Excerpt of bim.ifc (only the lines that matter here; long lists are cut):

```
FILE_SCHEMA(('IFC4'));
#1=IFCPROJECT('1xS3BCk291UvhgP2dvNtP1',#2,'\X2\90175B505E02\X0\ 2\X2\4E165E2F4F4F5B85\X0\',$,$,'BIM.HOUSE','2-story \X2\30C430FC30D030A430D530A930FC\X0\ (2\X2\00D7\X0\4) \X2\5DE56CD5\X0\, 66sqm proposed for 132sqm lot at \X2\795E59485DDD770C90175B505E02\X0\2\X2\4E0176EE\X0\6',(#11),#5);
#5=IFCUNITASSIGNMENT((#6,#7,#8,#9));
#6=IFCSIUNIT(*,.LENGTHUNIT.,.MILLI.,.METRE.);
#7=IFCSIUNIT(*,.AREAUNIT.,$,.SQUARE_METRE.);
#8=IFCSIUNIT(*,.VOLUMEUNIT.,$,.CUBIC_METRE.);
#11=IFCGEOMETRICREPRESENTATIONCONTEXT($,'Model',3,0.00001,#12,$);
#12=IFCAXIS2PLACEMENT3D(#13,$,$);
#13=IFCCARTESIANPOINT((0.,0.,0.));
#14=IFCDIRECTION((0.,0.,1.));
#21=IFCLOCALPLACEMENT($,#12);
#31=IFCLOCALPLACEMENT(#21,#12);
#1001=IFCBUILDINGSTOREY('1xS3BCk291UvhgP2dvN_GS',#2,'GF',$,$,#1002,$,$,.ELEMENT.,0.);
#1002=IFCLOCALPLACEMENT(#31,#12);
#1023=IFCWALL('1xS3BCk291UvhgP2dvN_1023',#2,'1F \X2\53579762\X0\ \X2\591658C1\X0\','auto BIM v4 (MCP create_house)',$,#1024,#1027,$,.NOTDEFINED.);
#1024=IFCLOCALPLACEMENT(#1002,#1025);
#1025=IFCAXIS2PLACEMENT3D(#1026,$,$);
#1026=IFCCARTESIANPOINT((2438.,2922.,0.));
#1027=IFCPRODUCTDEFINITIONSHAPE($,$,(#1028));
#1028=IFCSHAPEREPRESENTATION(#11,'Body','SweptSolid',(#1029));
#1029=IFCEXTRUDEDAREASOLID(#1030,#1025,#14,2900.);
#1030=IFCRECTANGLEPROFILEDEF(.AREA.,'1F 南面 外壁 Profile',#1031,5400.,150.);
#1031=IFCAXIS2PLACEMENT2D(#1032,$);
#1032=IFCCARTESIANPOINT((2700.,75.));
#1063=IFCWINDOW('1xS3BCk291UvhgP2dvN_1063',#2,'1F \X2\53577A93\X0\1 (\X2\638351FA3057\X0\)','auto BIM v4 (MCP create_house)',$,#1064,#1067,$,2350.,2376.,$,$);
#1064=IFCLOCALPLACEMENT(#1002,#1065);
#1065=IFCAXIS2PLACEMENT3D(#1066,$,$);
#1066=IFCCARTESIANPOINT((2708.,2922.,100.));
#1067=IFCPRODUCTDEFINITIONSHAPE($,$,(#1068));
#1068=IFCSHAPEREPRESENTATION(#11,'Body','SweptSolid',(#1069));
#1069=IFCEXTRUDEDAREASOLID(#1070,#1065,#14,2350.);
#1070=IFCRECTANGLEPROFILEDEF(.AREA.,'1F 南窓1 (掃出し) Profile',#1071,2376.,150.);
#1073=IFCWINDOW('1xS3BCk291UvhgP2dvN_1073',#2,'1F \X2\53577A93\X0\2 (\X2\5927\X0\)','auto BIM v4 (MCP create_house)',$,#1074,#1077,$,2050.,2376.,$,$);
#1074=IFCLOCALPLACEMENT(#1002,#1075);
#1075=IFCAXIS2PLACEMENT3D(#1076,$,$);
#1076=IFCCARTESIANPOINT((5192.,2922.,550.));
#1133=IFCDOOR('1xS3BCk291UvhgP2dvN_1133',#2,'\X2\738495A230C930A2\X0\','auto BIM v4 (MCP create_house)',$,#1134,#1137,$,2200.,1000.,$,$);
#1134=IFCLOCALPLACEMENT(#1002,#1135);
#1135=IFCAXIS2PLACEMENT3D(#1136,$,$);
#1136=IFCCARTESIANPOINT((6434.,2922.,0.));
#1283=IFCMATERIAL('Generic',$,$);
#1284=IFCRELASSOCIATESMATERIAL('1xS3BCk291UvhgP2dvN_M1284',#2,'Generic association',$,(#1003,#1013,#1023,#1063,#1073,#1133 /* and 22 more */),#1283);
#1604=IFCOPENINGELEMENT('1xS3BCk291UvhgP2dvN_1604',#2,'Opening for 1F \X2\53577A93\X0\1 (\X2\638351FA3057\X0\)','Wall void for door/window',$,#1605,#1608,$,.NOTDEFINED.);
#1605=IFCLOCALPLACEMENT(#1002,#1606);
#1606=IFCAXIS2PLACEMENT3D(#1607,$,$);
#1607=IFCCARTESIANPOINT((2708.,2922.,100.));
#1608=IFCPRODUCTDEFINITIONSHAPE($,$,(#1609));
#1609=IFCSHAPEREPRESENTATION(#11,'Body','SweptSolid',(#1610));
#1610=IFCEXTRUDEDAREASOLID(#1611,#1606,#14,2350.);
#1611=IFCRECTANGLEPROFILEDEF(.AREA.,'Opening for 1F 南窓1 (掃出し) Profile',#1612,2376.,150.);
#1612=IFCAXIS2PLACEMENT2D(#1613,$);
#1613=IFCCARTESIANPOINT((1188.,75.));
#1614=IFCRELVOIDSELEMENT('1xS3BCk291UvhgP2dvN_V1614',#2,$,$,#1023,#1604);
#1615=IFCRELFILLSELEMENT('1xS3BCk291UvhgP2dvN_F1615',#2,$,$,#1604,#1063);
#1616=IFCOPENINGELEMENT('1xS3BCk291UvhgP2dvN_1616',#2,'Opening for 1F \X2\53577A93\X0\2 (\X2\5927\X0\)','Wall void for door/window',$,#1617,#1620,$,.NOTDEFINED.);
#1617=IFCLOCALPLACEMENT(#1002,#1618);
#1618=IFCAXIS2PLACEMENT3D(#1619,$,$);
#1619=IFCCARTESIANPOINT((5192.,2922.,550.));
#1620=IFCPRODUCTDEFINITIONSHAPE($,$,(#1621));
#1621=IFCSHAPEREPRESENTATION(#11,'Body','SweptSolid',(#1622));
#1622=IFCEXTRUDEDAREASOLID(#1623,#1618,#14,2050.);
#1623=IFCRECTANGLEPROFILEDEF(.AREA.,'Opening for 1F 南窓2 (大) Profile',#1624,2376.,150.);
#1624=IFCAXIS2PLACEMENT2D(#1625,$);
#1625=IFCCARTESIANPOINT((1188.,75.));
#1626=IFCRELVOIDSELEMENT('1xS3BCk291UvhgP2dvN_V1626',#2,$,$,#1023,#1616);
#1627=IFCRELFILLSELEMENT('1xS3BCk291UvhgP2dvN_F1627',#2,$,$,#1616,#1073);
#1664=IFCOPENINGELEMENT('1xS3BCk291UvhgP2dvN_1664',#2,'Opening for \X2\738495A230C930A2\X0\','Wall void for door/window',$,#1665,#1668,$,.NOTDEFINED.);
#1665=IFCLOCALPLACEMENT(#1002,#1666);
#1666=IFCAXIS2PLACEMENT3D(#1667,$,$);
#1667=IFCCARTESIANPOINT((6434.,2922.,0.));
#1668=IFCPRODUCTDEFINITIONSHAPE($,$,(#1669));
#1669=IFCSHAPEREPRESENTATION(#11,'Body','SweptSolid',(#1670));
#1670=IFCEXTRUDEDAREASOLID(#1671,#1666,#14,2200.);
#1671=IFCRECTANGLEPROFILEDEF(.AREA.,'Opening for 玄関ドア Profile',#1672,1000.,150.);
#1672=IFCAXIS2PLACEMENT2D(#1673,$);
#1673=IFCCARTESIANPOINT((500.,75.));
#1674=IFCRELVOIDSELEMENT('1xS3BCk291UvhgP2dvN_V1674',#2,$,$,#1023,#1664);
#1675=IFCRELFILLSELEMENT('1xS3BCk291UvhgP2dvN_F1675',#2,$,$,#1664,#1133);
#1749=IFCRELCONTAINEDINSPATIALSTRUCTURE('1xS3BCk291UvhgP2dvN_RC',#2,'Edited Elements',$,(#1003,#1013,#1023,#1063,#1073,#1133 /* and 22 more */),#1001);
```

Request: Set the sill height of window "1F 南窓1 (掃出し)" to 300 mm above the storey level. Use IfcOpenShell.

```python
import numpy as np
import ifcopenshell
import ifcopenshell.api.geometry
import ifcopenshell.geom
import ifcopenshell.util.element
import ifcopenshell.util.placement
import ifcopenshell.util.shape
import ifcopenshell.util.unit

model = ifcopenshell.open("bim.ifc")
unit_scale = ifcopenshell.util.unit.calculate_unit_scale(model)

window = model.by_guid("1xS3BCk291UvhgP2dvN_1063")
opening = window.FillsVoids[0].RelatingOpeningElement
storey = ifcopenshell.util.element.get_container(window, ifc_class="IfcBuildingStorey")
level = ifcopenshell.util.placement.get_local_placement(storey.ObjectPlacement)[2, 3]

# The opening's origin need not be at the sill, so measure its lowest point.
shape = ifcopenshell.geom.create_shape(ifcopenshell.geom.settings(), opening)
bottom = ifcopenshell.util.shape.get_shape_bottom_elevation(shape, shape.geometry) / unit_scale
dz = level + 300.0 - bottom

shift = np.array([0.0, 0.0, dz])
# The window is not placed relative to its opening, so move both.
for product in (opening, window):
    matrix = ifcopenshell.util.placement.get_local_placement(product.ObjectPlacement)
    matrix[:3, 3] += shift
    ifcopenshell.api.geometry.edit_object_placement(model, product=product, matrix=matrix, is_si=False)

print(f"moved by {dz * unit_scale:+.3f} m")

model.write("bim_v2.ifc")
```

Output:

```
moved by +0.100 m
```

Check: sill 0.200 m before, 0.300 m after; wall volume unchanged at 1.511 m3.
